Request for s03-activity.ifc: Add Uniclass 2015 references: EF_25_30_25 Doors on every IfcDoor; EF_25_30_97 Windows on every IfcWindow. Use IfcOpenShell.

First a look at what the model holds.

```python
import ifcopenshell

model = ifcopenshell.open("s03-activity.ifc")
print(model.schema)
print("classifications:", [c.Name for c in model.by_type("IfcClassification")])
for ifc_class in ("IfcDoor", "IfcRoof", "IfcStair", "IfcWall", "IfcWindow"):
    print(ifc_class, len(model.by_type(ifc_class)))
```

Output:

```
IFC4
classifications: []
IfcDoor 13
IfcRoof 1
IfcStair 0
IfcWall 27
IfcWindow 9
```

```python
import ifcopenshell
import ifcopenshell.api.classification

model = ifcopenshell.open("s03-activity.ifc")

system = ifcopenshell.api.classification.add_classification(model, classification="Uniclass 2015")

codes = {
    "IfcDoor": ("EF_25_30_25", "Doors"),
    "IfcWindow": ("EF_25_30_97", "Windows"),
}
for ifc_class, (code, name) in codes.items():
    products = model.by_type(ifc_class)
    ifcopenshell.api.classification.add_reference(
        model, products=products, classification=system, identification=code, name=name
    )
    print(code, len(products))

model.write("s03-activity_updated.ifc")
```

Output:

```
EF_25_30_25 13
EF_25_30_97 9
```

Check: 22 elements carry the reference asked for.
